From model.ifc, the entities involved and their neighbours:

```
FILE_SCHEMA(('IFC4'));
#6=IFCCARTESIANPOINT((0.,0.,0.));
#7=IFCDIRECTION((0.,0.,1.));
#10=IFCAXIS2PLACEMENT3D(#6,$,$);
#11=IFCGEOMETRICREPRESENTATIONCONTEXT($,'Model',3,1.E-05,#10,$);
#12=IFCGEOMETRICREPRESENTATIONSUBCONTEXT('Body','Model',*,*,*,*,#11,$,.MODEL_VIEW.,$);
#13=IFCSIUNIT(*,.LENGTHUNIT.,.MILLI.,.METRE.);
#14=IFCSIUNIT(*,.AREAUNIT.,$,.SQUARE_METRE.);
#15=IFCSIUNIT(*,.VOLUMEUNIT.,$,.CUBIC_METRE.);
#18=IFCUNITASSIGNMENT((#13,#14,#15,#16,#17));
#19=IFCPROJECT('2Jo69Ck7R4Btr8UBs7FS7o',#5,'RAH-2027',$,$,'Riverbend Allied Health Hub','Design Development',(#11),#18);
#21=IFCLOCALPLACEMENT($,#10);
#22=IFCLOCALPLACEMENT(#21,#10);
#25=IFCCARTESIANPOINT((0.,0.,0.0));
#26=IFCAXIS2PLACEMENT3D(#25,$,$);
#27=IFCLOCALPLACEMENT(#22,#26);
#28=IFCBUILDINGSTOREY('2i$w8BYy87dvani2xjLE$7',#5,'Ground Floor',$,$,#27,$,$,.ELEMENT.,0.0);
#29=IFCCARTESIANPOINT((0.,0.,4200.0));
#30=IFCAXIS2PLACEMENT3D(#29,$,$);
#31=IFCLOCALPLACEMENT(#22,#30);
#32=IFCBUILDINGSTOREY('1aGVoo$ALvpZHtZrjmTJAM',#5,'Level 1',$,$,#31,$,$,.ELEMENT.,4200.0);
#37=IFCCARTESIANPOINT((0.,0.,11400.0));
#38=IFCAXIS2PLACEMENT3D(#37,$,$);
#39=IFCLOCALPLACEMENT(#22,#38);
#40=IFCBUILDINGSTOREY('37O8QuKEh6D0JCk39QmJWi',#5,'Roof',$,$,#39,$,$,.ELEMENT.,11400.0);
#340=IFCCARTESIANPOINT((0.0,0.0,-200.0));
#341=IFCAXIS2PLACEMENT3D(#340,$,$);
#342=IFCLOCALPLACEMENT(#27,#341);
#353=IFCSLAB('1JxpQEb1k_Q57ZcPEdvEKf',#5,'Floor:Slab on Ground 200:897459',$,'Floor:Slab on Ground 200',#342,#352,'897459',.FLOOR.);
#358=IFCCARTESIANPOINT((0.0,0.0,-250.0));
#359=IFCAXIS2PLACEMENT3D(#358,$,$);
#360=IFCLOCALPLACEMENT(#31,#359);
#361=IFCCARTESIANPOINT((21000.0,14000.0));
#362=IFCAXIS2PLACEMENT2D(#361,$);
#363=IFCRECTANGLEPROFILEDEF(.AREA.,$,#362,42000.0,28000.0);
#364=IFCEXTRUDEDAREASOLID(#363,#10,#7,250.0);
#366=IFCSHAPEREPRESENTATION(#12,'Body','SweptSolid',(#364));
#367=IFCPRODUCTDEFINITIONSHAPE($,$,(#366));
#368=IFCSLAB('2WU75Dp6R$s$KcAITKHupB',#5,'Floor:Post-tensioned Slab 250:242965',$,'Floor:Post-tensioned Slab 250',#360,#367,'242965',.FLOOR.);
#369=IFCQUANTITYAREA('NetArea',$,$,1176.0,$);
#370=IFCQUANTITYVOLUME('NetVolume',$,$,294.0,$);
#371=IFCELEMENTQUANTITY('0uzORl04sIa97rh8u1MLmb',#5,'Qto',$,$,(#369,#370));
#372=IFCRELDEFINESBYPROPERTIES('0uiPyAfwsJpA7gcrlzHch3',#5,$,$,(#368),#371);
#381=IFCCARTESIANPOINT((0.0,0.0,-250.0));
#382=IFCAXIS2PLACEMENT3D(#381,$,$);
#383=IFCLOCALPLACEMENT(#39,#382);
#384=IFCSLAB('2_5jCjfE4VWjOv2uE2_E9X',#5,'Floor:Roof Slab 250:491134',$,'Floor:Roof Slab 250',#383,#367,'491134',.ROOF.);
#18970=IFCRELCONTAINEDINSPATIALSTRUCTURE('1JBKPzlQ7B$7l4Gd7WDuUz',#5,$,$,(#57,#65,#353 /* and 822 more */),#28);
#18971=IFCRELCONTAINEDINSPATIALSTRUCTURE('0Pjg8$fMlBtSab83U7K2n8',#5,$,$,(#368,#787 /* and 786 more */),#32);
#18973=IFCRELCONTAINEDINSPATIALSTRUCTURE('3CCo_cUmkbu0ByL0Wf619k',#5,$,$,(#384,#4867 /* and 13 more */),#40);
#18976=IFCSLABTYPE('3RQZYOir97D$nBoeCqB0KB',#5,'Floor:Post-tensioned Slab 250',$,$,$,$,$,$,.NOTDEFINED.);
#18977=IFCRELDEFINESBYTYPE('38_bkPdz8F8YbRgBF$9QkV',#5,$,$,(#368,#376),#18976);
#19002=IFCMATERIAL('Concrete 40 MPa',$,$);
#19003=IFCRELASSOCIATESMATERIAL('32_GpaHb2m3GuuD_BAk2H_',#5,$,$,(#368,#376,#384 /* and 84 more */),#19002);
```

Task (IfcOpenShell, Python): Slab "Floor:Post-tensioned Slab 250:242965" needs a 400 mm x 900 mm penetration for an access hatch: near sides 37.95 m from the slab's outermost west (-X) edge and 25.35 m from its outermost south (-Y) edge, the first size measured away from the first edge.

```python
import numpy as np
import ifcopenshell
import ifcopenshell.api.feature
import ifcopenshell.api.geometry
import ifcopenshell.api.pset
import ifcopenshell.api.root
import ifcopenshell.geom
import ifcopenshell.util.element
import ifcopenshell.util.placement
import ifcopenshell.util.representation
import ifcopenshell.util.shape
import ifcopenshell.util.unit

model = ifcopenshell.open("model.ifc")
unit_scale = ifcopenshell.util.unit.calculate_unit_scale(model)
area_scale = ifcopenshell.util.unit.calculate_unit_scale(model, "AREAUNIT")
volume_scale = ifcopenshell.util.unit.calculate_unit_scale(model, "VOLUMEUNIT")
settings = ifcopenshell.geom.settings()


def volume(element):
    """Net volume in cubic metres, openings subtracted."""
    shape = ifcopenshell.geom.create_shape(settings, element)
    return ifcopenshell.util.shape.get_volume(shape.geometry)


slab = model.by_id(368)
before = volume(slab)

# Extent in the slab's own axes, in metres. The edges named are its -X and -Y sides.
slab_shape = ifcopenshell.geom.create_shape(settings, slab)
vertices = ifcopenshell.util.shape.get_vertices(slab_shape.geometry)
x_min, y_min, bottom = vertices.min(axis=0)
top = vertices[:, 2].max()

opening = ifcopenshell.api.root.create_entity(model, ifc_class="IfcOpeningElement", name="Access hatch opening", predefined_type="OPENING")
context = ifcopenshell.util.representation.get_context(model, "Model", "Body", "MODEL_VIEW")
width, depth = 0.4, 0.9
outline = [(0.0, 0.0), (width, 0.0), (width, depth), (0.0, depth), (0.0, 0.0)]
# Overshoot both faces by 50 mm so the cut is clean.
shape = ifcopenshell.api.geometry.add_slab_representation(
    model, context=context, depth=top - bottom + 0.1, polyline=outline
)
ifcopenshell.api.geometry.assign_representation(model, product=opening, representation=shape)

matrix = ifcopenshell.util.placement.get_local_placement(slab.ObjectPlacement)
matrix[:, 3] = matrix @ np.append(np.array([x_min + 37.95, y_min + 25.35, bottom - 0.05]) / unit_scale, 1.0)
ifcopenshell.api.geometry.edit_object_placement(model, product=opening, matrix=matrix, is_si=False)
ifcopenshell.api.feature.add_feature(model, feature=opening, element=slab)

after = volume(slab)

# Update the slab's stored quantities.
qto = model.by_id(ifcopenshell.util.element.get_pset(slab, "Qto", should_inherit=False)["id"])
ifcopenshell.api.pset.edit_qto(model, qto=qto, properties={
    "NetArea": after / (top - bottom) / area_scale,
    "NetVolume": after / volume_scale,
})

print(f"slab volume {before:.3f} -> {after:.3f} m3")

model.write("model_updated.ifc")
```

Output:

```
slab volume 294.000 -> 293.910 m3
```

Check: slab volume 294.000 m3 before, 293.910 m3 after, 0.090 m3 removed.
